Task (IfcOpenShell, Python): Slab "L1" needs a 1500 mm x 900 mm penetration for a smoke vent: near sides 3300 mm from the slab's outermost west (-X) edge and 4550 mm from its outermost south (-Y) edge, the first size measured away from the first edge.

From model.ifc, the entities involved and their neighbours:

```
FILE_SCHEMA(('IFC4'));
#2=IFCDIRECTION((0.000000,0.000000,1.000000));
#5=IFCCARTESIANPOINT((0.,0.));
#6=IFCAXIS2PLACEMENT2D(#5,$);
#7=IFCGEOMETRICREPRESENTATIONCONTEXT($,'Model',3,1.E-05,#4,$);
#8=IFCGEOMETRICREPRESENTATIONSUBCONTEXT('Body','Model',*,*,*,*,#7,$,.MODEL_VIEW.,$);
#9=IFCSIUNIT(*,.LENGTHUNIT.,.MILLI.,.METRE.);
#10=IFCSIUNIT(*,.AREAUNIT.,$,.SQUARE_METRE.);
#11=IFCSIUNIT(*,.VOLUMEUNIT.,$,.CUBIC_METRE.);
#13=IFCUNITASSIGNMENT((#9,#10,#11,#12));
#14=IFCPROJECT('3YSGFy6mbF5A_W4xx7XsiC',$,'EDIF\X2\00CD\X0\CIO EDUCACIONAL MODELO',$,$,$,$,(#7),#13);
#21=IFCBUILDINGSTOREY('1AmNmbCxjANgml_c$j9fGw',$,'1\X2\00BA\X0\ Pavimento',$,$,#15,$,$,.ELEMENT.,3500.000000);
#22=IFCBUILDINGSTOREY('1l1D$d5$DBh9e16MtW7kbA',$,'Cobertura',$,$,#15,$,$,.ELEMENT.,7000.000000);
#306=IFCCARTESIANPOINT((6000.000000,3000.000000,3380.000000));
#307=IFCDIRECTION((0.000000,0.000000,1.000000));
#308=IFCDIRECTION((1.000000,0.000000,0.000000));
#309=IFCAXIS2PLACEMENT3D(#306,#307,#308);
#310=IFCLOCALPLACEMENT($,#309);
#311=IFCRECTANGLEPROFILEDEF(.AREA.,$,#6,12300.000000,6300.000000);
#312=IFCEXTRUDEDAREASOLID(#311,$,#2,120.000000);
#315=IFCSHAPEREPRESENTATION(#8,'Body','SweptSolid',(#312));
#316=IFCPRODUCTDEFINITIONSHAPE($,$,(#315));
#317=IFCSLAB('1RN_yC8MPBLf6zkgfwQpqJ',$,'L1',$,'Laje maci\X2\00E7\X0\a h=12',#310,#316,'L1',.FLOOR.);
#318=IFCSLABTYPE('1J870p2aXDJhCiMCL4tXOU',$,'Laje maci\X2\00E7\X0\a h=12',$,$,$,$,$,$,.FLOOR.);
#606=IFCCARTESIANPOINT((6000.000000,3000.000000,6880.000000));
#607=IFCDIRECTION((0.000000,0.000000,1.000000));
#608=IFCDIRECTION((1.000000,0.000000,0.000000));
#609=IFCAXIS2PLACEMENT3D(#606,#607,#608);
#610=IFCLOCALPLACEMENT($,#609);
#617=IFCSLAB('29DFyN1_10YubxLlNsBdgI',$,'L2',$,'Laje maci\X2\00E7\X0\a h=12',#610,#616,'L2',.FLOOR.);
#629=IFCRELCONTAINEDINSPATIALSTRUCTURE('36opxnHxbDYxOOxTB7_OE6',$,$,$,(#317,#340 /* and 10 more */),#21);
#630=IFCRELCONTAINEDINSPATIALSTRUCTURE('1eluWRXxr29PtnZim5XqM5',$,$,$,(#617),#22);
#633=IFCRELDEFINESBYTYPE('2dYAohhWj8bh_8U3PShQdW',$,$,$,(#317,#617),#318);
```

```python
import numpy as np
import ifcopenshell
import ifcopenshell.api.feature
import ifcopenshell.api.geometry
import ifcopenshell.api.root
import ifcopenshell.geom
import ifcopenshell.util.placement
import ifcopenshell.util.representation
import ifcopenshell.util.shape
import ifcopenshell.util.unit

model = ifcopenshell.open("model.ifc")
unit_scale = ifcopenshell.util.unit.calculate_unit_scale(model)
settings = ifcopenshell.geom.settings()


def volume(element):
    """Net volume in cubic metres, openings subtracted."""
    shape = ifcopenshell.geom.create_shape(settings, element)
    return ifcopenshell.util.shape.get_volume(shape.geometry)


slab = model.by_id(317)
before = volume(slab)

# Extent in the slab's own axes, in metres. The edges named are its -X and -Y sides.
slab_shape = ifcopenshell.geom.create_shape(settings, slab)
vertices = ifcopenshell.util.shape.get_vertices(slab_shape.geometry)
x_min, y_min, bottom = vertices.min(axis=0)
top = vertices[:, 2].max()

opening = ifcopenshell.api.root.create_entity(model, ifc_class="IfcOpeningElement", name="Smoke vent opening", predefined_type="OPENING")
context = ifcopenshell.util.representation.get_context(model, "Model", "Body", "MODEL_VIEW")
width, depth = 1.5, 0.9
outline = [(0.0, 0.0), (width, 0.0), (width, depth), (0.0, depth), (0.0, 0.0)]
# Overshoot both faces by 50 mm so the cut is clean.
shape = ifcopenshell.api.geometry.add_slab_representation(
    model, context=context, depth=top - bottom + 0.1, polyline=outline
)
ifcopenshell.api.geometry.assign_representation(model, product=opening, representation=shape)

matrix = ifcopenshell.util.placement.get_local_placement(slab.ObjectPlacement)
matrix[:, 3] = matrix @ np.append(np.array([x_min + 3.3, y_min + 4.55, bottom - 0.05]) / unit_scale, 1.0)
ifcopenshell.api.geometry.edit_object_placement(model, product=opening, matrix=matrix, is_si=False)
ifcopenshell.api.feature.add_feature(model, feature=opening, element=slab)

after = volume(slab)

print(f"slab volume {before:.3f} -> {after:.3f} m3")

model.write("model_rev.ifc")
```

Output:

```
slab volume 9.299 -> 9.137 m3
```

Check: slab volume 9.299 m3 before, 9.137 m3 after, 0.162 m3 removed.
